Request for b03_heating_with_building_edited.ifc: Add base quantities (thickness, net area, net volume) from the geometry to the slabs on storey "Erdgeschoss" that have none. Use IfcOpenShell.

First a look at what the model holds.

```python
import ifcopenshell
import ifcopenshell.util.element
import ifcopenshell.util.unit

model = ifcopenshell.open("b03_heating_with_building_edited.ifc")
print(model.schema)
for unit_type in ("LENGTHUNIT", "AREAUNIT", "VOLUMEUNIT"):
    print(unit_type, ifcopenshell.util.unit.calculate_unit_scale(model, unit_type))
storey = next(s for s in model.by_type("IfcBuildingStorey") if s.Name == "Erdgeschoss")
slabs = [e for e in ifcopenshell.util.element.get_decomposition(storey) if e.is_a("IfcSlab")]
for e in sorted(slabs, key=lambda e: e.id()):
    print(e.id(), e.is_a(), e.Name, list(ifcopenshell.util.element.get_psets(e, qtos_only=True)), sep=" | ")
```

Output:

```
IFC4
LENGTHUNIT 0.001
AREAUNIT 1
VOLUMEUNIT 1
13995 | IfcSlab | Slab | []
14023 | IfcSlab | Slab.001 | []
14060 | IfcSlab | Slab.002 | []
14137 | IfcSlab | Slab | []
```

```python
import ifcopenshell
import ifcopenshell.api.pset
import ifcopenshell.geom
import ifcopenshell.util.element
import ifcopenshell.util.shape
import ifcopenshell.util.unit

model = ifcopenshell.open("b03_heating_with_building_edited.ifc")
unit_scale = ifcopenshell.util.unit.calculate_unit_scale(model)
area_scale = ifcopenshell.util.unit.calculate_unit_scale(model, "AREAUNIT")
volume_scale = ifcopenshell.util.unit.calculate_unit_scale(model, "VOLUMEUNIT")
settings = ifcopenshell.geom.settings()

storey = next(s for s in model.by_type("IfcBuildingStorey") if s.Name == "Erdgeschoss")
slabs = [e for e in ifcopenshell.util.element.get_decomposition(storey) if e.is_a("IfcSlab")]

for e in sorted(slabs, key=lambda e: e.id()):
    if ifcopenshell.util.element.get_psets(e, qtos_only=True, should_inherit=False):
        continue
    # Geometry comes back in metres, in the element's own axes.
    shape = ifcopenshell.geom.create_shape(settings, e)
    values = {
        "Width": ifcopenshell.util.shape.get_z(shape.geometry) / unit_scale,
        "NetArea": ifcopenshell.util.shape.get_footprint_area(shape.geometry) / area_scale,
        "NetVolume": ifcopenshell.util.shape.get_volume(shape.geometry) / volume_scale,
    }
    qto = ifcopenshell.api.pset.add_qto(model, product=e, name="Qto_SlabBaseQuantities")
    ifcopenshell.api.pset.edit_qto(model, qto=qto, properties=values)
    print(e.id(), {k: round(v, 3) for k, v in values.items()})

model.write("b03_heating_with_building_edited-out.ifc")
```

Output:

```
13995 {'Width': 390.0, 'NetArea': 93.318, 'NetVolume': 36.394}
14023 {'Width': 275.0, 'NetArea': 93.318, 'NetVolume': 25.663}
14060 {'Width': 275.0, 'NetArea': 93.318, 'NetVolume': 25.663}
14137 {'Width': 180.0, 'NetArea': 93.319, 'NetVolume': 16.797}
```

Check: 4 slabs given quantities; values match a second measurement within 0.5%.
